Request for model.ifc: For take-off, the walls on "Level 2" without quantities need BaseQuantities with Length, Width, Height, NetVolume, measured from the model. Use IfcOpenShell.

First a look at what the model holds.

```python
import ifcopenshell
import ifcopenshell.util.element
import ifcopenshell.util.unit

model = ifcopenshell.open("model.ifc")
print(model.schema)
for unit_type in ("LENGTHUNIT", "AREAUNIT", "VOLUMEUNIT"):
    print(unit_type, ifcopenshell.util.unit.calculate_unit_scale(model, unit_type))
storey = next(s for s in model.by_type("IfcBuildingStorey") if s.Name == "Level 2")
walls = [e for e in ifcopenshell.util.element.get_decomposition(storey) if e.is_a("IfcWall")]
for e in sorted(walls, key=lambda e: e.id()):
    print(e.id(), e.is_a(), e.Name, list(ifcopenshell.util.element.get_psets(e, qtos_only=True)), sep=" | ")
```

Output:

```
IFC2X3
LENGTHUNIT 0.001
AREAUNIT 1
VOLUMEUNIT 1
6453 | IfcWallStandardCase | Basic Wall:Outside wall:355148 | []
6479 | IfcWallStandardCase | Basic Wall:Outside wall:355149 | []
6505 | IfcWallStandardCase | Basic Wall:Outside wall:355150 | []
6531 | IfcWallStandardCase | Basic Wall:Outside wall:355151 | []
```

```python
import ifcopenshell
import ifcopenshell.api.pset
import ifcopenshell.geom
import ifcopenshell.util.element
import ifcopenshell.util.shape
import ifcopenshell.util.unit

model = ifcopenshell.open("model.ifc")
unit_scale = ifcopenshell.util.unit.calculate_unit_scale(model)
volume_scale = ifcopenshell.util.unit.calculate_unit_scale(model, "VOLUMEUNIT")
settings = ifcopenshell.geom.settings()

storey = next(s for s in model.by_type("IfcBuildingStorey") if s.Name == "Level 2")
walls = [e for e in ifcopenshell.util.element.get_decomposition(storey) if e.is_a("IfcWall")]

for e in sorted(walls, key=lambda e: e.id()):
    if ifcopenshell.util.element.get_psets(e, qtos_only=True, should_inherit=False):
        continue
    # Geometry comes back in metres, in the element's own axes.
    shape = ifcopenshell.geom.create_shape(settings, e)
    values = {
        "Length": ifcopenshell.util.shape.get_x(shape.geometry) / unit_scale,
        "Width": ifcopenshell.util.shape.get_y(shape.geometry) / unit_scale,
        "Height": ifcopenshell.util.shape.get_z(shape.geometry) / unit_scale,
        "NetVolume": ifcopenshell.util.shape.get_volume(shape.geometry) / volume_scale,
    }
    qto = ifcopenshell.api.pset.add_qto(model, product=e, name="BaseQuantities")
    ifcopenshell.api.pset.edit_qto(model, qto=qto, properties=values)
    print(e.id(), {k: round(v, 3) for k, v in values.items()})

model.write("model_edited.ifc")
```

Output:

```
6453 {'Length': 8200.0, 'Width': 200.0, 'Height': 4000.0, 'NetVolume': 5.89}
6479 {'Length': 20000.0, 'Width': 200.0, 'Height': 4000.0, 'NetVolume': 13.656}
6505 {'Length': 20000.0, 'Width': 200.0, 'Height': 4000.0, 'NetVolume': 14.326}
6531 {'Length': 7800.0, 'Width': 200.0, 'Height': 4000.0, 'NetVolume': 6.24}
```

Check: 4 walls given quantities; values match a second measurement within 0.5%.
